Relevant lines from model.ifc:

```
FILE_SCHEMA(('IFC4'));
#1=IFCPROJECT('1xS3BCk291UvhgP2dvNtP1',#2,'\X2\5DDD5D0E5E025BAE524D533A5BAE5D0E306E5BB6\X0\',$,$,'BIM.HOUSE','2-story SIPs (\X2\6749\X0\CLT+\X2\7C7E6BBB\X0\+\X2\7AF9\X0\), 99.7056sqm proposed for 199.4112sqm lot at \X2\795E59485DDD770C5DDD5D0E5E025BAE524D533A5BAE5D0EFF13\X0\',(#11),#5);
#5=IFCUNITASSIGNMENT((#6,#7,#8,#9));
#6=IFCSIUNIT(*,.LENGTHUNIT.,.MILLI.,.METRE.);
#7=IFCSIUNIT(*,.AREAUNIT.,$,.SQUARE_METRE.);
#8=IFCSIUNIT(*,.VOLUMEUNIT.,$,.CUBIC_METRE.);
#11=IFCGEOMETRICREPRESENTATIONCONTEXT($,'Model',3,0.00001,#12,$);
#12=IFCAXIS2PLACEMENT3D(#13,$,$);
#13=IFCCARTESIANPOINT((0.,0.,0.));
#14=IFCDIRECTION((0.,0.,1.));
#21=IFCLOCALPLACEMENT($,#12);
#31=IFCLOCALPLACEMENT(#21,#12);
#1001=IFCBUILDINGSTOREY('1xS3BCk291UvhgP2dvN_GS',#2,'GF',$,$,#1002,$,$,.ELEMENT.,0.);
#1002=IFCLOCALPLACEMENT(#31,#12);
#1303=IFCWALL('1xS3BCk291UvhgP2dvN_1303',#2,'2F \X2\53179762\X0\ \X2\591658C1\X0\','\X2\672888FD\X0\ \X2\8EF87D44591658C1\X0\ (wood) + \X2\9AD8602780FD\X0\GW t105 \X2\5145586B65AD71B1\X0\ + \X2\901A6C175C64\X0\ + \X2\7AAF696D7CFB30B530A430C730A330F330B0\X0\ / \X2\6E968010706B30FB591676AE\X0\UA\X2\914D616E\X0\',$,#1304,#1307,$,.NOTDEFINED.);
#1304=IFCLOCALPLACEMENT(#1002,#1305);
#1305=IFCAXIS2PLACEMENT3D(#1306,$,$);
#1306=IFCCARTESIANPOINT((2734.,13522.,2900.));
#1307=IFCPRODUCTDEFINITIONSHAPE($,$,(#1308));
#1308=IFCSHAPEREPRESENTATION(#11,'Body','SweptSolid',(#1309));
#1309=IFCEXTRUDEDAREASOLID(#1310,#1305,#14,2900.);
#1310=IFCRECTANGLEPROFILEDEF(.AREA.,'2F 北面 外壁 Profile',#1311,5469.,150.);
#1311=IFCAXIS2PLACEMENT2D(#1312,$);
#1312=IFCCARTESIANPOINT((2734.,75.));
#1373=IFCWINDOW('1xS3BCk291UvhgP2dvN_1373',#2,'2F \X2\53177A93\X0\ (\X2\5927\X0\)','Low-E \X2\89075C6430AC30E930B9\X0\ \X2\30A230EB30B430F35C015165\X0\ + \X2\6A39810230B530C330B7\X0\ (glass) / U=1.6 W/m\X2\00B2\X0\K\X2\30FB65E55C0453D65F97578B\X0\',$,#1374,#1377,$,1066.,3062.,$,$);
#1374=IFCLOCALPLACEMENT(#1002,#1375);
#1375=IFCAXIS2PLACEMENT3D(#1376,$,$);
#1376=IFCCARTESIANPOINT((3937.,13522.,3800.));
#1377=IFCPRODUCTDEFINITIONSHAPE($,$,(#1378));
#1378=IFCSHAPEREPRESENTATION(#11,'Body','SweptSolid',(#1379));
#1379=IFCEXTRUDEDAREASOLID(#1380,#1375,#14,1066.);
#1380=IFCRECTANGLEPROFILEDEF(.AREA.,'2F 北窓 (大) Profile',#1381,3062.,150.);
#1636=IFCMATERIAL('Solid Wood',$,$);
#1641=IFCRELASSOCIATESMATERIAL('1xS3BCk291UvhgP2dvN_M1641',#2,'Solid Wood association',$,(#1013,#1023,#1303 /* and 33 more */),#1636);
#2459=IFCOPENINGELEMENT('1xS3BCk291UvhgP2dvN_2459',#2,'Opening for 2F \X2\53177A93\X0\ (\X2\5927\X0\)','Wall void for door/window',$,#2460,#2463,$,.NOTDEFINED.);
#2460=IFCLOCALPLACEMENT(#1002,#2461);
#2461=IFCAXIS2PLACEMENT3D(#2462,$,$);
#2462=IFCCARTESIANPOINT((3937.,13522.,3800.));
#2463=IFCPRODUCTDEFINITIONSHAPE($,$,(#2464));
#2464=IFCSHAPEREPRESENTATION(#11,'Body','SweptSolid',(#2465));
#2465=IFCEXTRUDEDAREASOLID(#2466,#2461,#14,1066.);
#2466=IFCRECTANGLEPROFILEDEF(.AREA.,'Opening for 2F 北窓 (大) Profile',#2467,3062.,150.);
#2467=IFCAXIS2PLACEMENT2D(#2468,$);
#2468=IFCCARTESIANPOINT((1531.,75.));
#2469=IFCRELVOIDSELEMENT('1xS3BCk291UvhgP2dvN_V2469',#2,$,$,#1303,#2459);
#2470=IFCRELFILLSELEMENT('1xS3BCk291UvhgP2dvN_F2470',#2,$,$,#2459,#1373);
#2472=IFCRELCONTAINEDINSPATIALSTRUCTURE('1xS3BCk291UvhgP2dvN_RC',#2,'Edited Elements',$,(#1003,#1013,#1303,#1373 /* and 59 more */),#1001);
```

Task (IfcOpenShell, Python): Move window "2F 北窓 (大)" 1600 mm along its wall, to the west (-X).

```python
import ifcopenshell
import ifcopenshell.api.geometry
import ifcopenshell.util.placement
import ifcopenshell.util.unit

model = ifcopenshell.open("model.ifc")
unit_scale = ifcopenshell.util.unit.calculate_unit_scale(model)

window = model.by_guid("1xS3BCk291UvhgP2dvN_1373")
opening = window.FillsVoids[0].RelatingOpeningElement
wall = opening.VoidsElements[0].RelatingBuildingElement

wall_matrix = ifcopenshell.util.placement.get_local_placement(wall.ObjectPlacement)
shift = wall_matrix[:3, 0] * -1.6 / unit_scale
before = ifcopenshell.util.placement.get_local_placement(window.ObjectPlacement)[:3, 3].copy()

# The window is not placed relative to its opening, so move both.
for product in (opening, window):
    matrix = ifcopenshell.util.placement.get_local_placement(product.ObjectPlacement)
    matrix[:3, 3] += shift
    ifcopenshell.api.geometry.edit_object_placement(model, product=product, matrix=matrix, is_si=False)

after = ifcopenshell.util.placement.get_local_placement(window.ObjectPlacement)[:3, 3]
print("window moved by", (after - before).round(3) + 0.0)

model.write("model_updated.ifc")
```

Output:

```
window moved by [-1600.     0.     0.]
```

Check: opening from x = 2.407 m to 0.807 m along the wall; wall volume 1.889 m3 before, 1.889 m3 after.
